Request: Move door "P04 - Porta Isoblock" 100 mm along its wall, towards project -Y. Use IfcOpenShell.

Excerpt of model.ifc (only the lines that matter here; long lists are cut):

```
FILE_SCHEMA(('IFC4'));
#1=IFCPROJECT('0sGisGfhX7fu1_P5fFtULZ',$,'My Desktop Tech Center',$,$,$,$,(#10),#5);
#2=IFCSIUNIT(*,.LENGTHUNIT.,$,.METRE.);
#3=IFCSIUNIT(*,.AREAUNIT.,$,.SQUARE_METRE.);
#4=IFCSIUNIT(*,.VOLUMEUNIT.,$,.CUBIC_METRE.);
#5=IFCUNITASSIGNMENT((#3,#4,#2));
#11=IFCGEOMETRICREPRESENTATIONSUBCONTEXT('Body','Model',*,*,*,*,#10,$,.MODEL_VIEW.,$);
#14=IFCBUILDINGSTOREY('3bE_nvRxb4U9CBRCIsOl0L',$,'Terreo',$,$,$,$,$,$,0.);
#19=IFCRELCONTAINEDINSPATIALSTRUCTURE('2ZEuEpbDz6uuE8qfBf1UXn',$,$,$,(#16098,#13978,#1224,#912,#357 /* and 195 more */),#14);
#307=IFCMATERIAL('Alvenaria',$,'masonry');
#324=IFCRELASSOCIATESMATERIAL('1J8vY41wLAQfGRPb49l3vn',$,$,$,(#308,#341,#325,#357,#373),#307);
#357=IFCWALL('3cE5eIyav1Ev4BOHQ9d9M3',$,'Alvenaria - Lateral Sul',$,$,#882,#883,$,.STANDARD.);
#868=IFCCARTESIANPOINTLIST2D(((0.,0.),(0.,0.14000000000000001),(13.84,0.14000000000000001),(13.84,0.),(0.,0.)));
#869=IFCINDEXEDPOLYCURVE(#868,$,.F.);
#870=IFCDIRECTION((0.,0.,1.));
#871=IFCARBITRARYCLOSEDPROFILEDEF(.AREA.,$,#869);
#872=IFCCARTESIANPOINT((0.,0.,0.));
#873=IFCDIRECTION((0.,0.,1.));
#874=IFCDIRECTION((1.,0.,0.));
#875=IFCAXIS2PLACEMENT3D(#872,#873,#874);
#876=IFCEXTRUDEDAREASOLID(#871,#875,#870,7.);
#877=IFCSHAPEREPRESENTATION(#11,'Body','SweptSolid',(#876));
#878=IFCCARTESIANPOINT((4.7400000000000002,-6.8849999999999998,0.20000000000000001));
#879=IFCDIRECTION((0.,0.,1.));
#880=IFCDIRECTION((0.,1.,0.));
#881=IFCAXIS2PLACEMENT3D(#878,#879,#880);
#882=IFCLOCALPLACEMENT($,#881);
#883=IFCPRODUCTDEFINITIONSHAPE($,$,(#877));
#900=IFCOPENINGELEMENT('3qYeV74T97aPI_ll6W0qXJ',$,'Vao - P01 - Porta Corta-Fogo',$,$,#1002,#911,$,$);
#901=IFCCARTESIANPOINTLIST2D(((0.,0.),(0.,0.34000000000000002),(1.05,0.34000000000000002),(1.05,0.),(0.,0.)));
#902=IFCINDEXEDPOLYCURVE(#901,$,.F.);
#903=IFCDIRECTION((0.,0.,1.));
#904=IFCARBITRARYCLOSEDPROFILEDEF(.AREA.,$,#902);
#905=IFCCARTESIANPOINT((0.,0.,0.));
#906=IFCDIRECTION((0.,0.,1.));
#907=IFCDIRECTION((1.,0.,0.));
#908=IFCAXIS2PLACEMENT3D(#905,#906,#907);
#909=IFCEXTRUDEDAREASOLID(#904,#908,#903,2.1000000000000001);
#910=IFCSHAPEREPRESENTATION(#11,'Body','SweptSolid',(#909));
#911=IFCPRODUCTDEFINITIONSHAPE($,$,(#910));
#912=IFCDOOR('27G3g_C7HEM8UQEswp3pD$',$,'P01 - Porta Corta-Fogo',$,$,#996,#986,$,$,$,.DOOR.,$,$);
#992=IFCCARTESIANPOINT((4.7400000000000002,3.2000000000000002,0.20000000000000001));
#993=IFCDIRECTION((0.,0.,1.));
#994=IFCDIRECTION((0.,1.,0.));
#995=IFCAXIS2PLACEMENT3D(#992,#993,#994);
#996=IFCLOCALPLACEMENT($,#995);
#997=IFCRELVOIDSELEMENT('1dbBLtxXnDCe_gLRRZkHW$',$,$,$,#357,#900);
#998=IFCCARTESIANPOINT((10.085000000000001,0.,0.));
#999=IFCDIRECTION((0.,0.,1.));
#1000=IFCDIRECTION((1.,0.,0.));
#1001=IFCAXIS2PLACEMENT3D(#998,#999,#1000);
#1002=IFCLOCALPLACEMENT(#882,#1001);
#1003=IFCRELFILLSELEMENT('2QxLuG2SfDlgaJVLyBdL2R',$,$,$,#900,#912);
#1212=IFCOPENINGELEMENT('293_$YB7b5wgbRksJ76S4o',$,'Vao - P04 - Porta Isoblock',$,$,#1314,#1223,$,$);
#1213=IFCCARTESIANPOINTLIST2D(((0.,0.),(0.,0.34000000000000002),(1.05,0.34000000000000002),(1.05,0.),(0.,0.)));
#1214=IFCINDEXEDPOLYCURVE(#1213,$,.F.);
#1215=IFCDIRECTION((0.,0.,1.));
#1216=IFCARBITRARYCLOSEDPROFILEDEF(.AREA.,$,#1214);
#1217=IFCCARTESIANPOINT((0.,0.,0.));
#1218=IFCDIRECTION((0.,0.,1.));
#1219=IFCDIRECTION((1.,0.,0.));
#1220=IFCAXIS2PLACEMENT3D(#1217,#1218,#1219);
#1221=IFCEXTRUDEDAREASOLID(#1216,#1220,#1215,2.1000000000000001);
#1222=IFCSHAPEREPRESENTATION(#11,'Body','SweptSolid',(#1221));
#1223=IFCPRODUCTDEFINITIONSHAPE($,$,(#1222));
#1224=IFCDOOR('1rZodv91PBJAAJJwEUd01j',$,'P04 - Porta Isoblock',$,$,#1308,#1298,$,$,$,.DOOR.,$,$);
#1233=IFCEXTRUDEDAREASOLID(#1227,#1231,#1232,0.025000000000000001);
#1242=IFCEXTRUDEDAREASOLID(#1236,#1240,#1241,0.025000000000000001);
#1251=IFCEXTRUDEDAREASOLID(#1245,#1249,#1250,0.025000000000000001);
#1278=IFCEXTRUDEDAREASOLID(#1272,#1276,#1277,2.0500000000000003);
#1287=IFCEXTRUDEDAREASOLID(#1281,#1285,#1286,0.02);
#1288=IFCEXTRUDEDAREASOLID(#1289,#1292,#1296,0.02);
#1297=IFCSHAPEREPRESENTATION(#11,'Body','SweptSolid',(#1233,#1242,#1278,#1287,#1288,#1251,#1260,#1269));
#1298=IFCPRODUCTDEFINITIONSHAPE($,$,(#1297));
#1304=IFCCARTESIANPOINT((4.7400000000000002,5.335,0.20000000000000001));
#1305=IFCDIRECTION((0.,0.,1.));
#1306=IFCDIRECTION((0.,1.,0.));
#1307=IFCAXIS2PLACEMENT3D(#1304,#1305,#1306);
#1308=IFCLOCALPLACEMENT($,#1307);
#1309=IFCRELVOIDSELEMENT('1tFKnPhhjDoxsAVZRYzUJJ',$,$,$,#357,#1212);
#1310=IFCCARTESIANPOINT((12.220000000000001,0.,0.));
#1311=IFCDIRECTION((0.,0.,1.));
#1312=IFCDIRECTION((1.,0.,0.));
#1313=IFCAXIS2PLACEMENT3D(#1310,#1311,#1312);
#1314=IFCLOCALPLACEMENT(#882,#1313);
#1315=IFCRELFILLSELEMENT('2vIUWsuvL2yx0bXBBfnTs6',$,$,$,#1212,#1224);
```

```python
import ifcopenshell
import ifcopenshell.api.geometry
import ifcopenshell.util.placement

model = ifcopenshell.open("model.ifc")

door = model.by_guid("1rZodv91PBJAAJJwEUd01j")
opening = door.FillsVoids[0].RelatingOpeningElement
wall = opening.VoidsElements[0].RelatingBuildingElement

wall_matrix = ifcopenshell.util.placement.get_local_placement(wall.ObjectPlacement)
shift = wall_matrix[:3, 0] * -0.1
before = ifcopenshell.util.placement.get_local_placement(door.ObjectPlacement)[:3, 3].copy()

# The door is not placed relative to its opening, so move both.
for product in (opening, door):
    matrix = ifcopenshell.util.placement.get_local_placement(product.ObjectPlacement)
    matrix[:3, 3] += shift
    ifcopenshell.api.geometry.edit_object_placement(model, product=product, matrix=matrix, is_si=False)

after = ifcopenshell.util.placement.get_local_placement(door.ObjectPlacement)[:3, 3]
print("door moved by", (after - before).round(3) + 0.0)

model.write("model_edited.ifc")
```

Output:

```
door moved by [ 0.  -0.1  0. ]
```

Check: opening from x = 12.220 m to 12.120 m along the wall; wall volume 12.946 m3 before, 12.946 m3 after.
